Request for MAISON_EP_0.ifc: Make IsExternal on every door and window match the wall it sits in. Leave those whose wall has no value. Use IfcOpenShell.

First a look at what the model holds.

```python
import ifcopenshell
import ifcopenshell.util.element

model = ifcopenshell.open("MAISON_EP_0.ifc")
print(model.schema)
seen = {}
for e in model.by_type("IfcDoor") + model.by_type("IfcWindow"):
    if not e.FillsVoids:
        continue
    host = e.FillsVoids[0].RelatingOpeningElement.VoidsElements[0].RelatingBuildingElement
    own = ifcopenshell.util.element.get_pset(e, f"Pset_{e.is_a()[3:].removesuffix('StandardCase')}Common", "IsExternal")
    wall = ifcopenshell.util.element.get_pset(host, "Pset_WallCommon", "IsExternal")
    seen[e.is_a(), own, wall] = seen.get((e.is_a(), own, wall), 0) + 1
for (cls, own, wall), count in sorted(seen.items(), key=str):
    print(count, cls, "IsExternal:", own, "| host wall:", wall)
```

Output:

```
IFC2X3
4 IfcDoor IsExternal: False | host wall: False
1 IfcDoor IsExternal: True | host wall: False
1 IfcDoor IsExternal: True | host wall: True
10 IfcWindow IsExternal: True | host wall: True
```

```python
import ifcopenshell
import ifcopenshell.api.pset
import ifcopenshell.util.element

model = ifcopenshell.open("MAISON_EP_0.ifc")

count = 0
for ifc_class, pset_name in (("IfcDoor", "Pset_DoorCommon"), ("IfcWindow", "Pset_WindowCommon")):
    for e in model.by_type(ifc_class):
        if not e.FillsVoids:
            continue
        host = e.FillsVoids[0].RelatingOpeningElement.VoidsElements[0].RelatingBuildingElement
        external = ifcopenshell.util.element.get_pset(host, "Pset_WallCommon", "IsExternal")
        if external is None or ifcopenshell.util.element.get_pset(e, pset_name, "IsExternal") == external:
            continue
        pset = ifcopenshell.api.pset.add_pset(model, product=e, name=pset_name)
        ifcopenshell.api.pset.edit_pset(model, pset=pset, properties={"IsExternal": external})
        count += 1

print(count, "updated")

model.write("MAISON_EP_0_rev.ifc")
```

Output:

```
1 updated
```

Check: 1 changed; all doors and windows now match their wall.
